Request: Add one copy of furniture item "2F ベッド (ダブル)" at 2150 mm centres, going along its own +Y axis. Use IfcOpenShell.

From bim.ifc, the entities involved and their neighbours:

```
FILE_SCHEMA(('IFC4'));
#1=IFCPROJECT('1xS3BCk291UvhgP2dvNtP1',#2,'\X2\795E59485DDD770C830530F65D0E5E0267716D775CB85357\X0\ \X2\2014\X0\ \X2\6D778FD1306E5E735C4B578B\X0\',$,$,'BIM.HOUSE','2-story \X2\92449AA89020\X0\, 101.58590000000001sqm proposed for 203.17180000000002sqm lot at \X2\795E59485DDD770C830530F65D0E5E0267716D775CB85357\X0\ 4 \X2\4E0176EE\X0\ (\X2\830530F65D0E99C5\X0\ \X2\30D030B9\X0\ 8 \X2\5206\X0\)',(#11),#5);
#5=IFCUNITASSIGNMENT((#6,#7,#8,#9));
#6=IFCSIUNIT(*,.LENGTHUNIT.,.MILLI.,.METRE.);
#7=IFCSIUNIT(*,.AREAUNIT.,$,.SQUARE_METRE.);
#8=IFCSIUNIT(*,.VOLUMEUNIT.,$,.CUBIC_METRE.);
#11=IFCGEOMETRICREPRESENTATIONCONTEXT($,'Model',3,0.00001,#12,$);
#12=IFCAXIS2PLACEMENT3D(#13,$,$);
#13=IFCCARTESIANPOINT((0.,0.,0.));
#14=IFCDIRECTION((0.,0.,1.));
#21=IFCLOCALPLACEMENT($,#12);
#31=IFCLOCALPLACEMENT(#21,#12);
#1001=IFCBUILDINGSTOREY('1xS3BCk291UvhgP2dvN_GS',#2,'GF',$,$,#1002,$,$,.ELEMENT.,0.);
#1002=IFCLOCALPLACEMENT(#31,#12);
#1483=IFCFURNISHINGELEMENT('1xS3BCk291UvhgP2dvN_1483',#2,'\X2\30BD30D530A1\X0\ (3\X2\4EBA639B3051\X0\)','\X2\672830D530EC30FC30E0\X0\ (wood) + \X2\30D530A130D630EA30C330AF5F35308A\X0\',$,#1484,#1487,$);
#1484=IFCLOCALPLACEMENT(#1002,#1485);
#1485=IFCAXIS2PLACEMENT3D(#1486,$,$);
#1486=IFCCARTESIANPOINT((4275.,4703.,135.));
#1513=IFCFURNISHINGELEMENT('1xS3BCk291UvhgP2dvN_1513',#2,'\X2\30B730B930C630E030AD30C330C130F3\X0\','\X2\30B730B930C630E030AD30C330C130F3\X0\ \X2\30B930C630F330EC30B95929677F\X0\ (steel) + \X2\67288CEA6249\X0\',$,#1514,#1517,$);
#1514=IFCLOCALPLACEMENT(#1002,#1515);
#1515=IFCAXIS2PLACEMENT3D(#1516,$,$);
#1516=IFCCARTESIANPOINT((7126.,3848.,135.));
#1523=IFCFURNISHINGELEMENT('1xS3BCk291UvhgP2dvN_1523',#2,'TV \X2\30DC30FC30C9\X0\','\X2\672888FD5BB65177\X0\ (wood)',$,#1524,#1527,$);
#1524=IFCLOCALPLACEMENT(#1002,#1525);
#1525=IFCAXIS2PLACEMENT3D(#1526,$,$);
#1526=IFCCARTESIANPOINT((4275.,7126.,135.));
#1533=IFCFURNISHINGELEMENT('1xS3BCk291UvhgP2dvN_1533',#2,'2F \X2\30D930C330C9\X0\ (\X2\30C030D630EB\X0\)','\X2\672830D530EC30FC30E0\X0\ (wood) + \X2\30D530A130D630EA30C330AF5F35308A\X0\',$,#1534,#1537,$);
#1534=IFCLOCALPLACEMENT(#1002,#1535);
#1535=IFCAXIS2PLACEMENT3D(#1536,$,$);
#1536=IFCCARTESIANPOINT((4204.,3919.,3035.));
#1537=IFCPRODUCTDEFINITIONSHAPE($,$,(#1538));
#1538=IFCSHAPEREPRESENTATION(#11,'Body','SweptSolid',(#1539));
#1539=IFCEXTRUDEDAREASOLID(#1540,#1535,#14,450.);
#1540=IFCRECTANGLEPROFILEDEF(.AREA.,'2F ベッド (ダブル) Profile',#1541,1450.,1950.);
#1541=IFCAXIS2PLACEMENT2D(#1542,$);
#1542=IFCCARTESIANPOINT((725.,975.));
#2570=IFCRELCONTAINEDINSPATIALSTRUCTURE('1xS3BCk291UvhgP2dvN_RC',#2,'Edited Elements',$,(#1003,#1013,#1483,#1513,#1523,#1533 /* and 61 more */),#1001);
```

```python
import ifcopenshell
import ifcopenshell.api.geometry
import ifcopenshell.api.root
import ifcopenshell.util.element
import ifcopenshell.util.placement

model = ifcopenshell.open("bim.ifc")


def reuse_history(source, copy):
    """copy_class also copies each property set's owner history, people and application; keep the originals."""
    for rel in copy.IsDefinedBy:
        if rel.is_a("IfcRelDefinesByProperties") and (history := rel.RelatingPropertyDefinition.OwnerHistory):
            rel.RelatingPropertyDefinition.OwnerHistory = source.OwnerHistory
            ifcopenshell.util.element.remove_deep2(model, history)


source = model.by_guid("1xS3BCk291UvhgP2dvN_1533")
base = ifcopenshell.util.placement.get_local_placement(source.ObjectPlacement)
step = base[:3, 1] * 2150.0

for i in range(1, 2):
    copy = ifcopenshell.api.root.copy_class(model, product=source)
    copy.Representation = ifcopenshell.util.element.copy_deep(
        model, source.Representation, exclude=["IfcGeometricRepresentationContext", "IfcRepresentationMap"]
    )
    reuse_history(source, copy)
    matrix = base.copy()
    matrix[:3, 3] += i * step
    print("added at", matrix[:3, 3].round(3) + 0.0)
    ifcopenshell.api.geometry.edit_object_placement(model, product=copy, matrix=matrix, is_si=False)

model.write("bim_updated.ifc")
```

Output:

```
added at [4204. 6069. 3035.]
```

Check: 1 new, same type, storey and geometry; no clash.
